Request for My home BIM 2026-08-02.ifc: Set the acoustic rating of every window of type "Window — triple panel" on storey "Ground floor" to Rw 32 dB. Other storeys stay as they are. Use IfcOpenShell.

First a look at what the model holds.

```python
import ifcopenshell
import ifcopenshell.util.element

model = ifcopenshell.open("My home BIM 2026-08-02.ifc")
print(model.schema)
storey = next(s for s in model.by_type("IfcBuildingStorey") if s.Name == "Ground floor")
windows = [e for e in ifcopenshell.util.element.get_decomposition(storey) if e.is_a("IfcWindow")]
seen = {}
for e in windows:
    element_type = ifcopenshell.util.element.get_type(e)
    key = (element_type.Name if element_type != e and element_type else None, ifcopenshell.util.element.get_pset(e, "Pset_WindowCommon", "AcousticRating"))
    seen[key] = seen.get(key, 0) + 1
for (name, value), count in sorted(seen.items(), key=str):
    print(count, "x", name, "|", value)
```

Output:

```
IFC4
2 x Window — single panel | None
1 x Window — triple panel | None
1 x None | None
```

```python
import ifcopenshell
import ifcopenshell.api.pset
import ifcopenshell.util.element

model = ifcopenshell.open("My home BIM 2026-08-02.ifc")

storey = next(s for s in model.by_type("IfcBuildingStorey") if s.Name == "Ground floor")
windows = [e for e in ifcopenshell.util.element.get_decomposition(storey) if e.is_a("IfcWindow")]

count = 0
for e in windows:
    element_type = ifcopenshell.util.element.get_type(e)
    if element_type in (None, e) or element_type.Name != "Window — triple panel":
        continue
    # add_pset returns the element's existing set when there is one.
    pset = ifcopenshell.api.pset.add_pset(model, product=e, name="Pset_WindowCommon")
    ifcopenshell.api.pset.edit_pset(model, pset=pset, properties={"AcousticRating": "Rw 32 dB"})
    count += 1

print(count, "windows updated")

model.write("My home BIM 2026-08-02_v2.ifc")
```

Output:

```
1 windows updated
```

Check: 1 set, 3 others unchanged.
